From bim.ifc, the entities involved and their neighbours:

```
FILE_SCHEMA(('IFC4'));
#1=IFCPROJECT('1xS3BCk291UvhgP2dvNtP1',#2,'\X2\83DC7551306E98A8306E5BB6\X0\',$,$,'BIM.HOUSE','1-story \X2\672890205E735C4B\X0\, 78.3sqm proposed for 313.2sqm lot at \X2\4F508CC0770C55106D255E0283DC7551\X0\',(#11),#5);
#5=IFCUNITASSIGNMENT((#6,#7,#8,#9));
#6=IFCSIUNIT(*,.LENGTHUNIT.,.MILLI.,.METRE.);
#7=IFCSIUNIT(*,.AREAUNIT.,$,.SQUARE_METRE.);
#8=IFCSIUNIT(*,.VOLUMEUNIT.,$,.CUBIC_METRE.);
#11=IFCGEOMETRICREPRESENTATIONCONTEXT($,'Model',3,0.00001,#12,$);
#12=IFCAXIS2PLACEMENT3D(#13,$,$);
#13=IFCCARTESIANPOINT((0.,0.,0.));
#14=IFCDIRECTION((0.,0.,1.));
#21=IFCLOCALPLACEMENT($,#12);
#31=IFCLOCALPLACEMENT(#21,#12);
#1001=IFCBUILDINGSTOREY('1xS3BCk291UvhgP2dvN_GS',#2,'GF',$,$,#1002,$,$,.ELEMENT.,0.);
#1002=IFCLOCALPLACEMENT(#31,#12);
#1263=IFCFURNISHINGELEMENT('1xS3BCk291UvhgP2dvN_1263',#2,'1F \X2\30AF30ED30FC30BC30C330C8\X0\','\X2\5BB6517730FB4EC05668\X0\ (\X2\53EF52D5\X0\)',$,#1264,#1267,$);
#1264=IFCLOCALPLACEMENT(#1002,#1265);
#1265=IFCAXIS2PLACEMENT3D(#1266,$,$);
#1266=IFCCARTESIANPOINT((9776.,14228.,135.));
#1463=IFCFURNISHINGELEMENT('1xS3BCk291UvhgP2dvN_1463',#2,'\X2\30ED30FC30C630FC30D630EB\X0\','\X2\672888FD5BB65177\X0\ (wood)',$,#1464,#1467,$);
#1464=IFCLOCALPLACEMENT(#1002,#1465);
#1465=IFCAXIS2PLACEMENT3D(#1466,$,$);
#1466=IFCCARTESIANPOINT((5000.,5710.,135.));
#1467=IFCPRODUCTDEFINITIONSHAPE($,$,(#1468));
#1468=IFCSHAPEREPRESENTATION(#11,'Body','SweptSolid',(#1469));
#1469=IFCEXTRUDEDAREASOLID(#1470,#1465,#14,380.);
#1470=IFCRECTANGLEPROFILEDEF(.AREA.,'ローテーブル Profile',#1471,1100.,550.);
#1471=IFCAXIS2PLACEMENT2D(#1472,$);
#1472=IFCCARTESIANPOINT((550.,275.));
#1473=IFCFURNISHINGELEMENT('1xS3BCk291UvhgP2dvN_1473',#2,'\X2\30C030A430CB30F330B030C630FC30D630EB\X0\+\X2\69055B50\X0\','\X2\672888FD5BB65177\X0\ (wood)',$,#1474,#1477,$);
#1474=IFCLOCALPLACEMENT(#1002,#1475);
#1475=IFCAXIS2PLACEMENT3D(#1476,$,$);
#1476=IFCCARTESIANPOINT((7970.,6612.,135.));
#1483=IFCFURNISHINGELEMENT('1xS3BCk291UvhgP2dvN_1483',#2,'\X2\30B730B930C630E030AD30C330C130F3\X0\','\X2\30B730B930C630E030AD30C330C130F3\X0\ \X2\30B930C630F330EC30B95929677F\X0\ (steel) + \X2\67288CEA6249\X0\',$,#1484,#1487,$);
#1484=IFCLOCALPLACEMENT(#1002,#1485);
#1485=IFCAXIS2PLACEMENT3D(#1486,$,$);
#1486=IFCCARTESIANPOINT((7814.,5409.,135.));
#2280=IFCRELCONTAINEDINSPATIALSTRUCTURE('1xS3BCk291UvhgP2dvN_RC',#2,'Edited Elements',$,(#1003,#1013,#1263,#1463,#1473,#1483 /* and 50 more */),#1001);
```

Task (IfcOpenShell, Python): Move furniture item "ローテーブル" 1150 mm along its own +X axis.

```python
import ifcopenshell
import ifcopenshell.api.geometry
import ifcopenshell.util.placement

model = ifcopenshell.open("bim.ifc")

item = model.by_guid("1xS3BCk291UvhgP2dvN_1463")
matrix = ifcopenshell.util.placement.get_local_placement(item.ObjectPlacement)
matrix[:3, 3] += matrix[:3, 0] * 1150.0
ifcopenshell.api.geometry.edit_object_placement(model, product=item, matrix=matrix, is_si=False)

print(ifcopenshell.util.placement.get_local_placement(item.ObjectPlacement).round(3) + 0.0)

model.write("bim_v2.ifc")
```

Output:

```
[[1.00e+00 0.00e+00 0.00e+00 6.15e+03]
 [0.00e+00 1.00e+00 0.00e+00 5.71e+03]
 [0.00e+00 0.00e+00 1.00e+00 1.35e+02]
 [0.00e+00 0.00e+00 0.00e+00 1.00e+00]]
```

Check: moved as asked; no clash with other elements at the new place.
